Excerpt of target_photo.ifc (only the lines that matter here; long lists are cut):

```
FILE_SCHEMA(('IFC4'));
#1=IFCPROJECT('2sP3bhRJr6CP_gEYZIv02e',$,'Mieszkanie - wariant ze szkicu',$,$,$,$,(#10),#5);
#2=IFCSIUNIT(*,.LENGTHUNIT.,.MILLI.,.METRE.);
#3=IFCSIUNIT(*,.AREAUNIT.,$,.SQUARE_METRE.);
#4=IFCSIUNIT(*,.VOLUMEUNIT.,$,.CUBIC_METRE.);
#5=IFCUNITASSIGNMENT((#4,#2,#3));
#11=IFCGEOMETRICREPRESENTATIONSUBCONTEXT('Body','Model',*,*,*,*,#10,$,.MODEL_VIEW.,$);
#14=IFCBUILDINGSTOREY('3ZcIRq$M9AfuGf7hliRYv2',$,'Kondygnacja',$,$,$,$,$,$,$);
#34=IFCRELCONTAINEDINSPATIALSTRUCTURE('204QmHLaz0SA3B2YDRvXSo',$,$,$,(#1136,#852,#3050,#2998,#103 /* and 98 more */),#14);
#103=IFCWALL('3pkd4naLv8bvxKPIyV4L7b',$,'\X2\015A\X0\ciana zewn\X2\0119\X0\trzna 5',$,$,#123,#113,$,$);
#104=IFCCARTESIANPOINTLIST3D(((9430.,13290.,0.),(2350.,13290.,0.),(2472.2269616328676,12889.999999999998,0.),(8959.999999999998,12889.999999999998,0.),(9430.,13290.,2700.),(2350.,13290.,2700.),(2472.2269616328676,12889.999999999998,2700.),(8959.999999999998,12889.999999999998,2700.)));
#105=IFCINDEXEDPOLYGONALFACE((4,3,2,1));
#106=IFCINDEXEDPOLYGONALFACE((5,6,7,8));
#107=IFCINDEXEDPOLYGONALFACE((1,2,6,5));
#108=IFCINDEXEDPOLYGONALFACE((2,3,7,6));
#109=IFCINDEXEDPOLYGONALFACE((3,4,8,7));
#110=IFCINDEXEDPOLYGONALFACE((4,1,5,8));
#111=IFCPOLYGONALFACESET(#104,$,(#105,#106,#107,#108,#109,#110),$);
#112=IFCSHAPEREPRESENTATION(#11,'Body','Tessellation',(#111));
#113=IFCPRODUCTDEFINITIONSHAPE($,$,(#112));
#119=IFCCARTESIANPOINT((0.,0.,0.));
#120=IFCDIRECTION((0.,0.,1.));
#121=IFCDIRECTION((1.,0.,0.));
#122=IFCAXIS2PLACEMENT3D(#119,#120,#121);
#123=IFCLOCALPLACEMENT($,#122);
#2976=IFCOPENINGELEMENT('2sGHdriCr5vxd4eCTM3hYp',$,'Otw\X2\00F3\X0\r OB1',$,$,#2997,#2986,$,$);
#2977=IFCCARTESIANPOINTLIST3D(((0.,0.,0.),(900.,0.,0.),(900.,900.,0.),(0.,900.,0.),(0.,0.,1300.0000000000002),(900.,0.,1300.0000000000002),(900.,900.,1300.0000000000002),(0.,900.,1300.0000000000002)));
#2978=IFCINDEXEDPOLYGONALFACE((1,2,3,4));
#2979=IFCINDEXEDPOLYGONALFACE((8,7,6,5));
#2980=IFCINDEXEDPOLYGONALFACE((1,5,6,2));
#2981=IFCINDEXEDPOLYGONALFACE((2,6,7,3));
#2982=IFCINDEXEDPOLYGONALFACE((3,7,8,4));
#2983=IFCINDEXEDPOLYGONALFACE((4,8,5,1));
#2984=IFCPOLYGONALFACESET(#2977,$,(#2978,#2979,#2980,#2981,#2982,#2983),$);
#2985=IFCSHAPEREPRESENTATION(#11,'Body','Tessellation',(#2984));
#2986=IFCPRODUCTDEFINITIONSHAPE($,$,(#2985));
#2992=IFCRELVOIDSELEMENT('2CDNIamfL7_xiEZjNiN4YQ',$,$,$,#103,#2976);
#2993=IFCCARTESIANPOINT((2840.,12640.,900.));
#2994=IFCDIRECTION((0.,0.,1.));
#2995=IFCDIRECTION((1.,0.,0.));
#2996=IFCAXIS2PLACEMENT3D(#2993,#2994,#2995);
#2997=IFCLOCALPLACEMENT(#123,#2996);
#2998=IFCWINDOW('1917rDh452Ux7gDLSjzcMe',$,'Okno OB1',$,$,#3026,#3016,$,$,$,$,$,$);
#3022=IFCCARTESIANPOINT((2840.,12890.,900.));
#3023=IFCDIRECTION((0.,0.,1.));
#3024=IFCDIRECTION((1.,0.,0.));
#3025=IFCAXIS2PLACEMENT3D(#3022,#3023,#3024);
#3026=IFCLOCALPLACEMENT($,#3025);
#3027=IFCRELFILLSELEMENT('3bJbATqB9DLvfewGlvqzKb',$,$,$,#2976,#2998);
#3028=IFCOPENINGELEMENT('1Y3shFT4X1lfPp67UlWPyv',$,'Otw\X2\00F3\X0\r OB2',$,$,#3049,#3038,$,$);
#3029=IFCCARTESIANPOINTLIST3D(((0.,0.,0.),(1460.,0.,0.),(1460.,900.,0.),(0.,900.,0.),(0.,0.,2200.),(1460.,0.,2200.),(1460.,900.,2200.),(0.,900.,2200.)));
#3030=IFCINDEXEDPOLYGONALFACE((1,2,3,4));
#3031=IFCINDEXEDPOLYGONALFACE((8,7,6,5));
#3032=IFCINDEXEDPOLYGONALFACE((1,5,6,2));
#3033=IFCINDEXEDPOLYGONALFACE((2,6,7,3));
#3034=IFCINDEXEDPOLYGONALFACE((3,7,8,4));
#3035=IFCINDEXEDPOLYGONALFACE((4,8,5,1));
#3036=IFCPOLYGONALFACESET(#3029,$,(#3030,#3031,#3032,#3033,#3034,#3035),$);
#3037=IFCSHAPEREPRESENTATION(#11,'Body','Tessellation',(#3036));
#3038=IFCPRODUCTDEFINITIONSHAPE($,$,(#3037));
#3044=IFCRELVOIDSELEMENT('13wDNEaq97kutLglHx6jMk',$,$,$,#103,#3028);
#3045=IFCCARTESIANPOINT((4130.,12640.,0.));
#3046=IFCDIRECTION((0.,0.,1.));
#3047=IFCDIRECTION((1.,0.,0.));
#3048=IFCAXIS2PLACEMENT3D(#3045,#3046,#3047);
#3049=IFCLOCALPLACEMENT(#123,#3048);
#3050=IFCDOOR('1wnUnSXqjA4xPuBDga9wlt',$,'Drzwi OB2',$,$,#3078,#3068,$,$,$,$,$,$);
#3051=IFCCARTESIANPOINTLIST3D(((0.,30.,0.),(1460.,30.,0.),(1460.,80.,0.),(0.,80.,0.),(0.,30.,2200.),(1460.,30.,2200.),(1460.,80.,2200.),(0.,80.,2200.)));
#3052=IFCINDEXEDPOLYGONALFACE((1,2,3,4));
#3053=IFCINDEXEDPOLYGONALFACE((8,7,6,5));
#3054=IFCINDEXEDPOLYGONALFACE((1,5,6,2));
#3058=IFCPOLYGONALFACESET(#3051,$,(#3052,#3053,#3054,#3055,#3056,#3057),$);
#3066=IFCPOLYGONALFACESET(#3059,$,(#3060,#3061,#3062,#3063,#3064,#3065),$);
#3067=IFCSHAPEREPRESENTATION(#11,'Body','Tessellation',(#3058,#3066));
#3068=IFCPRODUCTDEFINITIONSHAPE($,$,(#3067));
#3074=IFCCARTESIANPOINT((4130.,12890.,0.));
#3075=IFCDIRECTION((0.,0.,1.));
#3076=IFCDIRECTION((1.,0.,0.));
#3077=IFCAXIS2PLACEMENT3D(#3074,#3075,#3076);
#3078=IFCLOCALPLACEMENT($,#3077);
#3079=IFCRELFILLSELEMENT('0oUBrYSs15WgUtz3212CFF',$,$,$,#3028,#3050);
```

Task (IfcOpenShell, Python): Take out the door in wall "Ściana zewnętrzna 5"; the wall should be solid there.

```python
import ifcopenshell
import ifcopenshell.api.feature
import ifcopenshell.api.root
import ifcopenshell.geom
import ifcopenshell.util.shape

model = ifcopenshell.open("target_photo.ifc")
settings = ifcopenshell.geom.settings()


def volume(element):
    """Net volume in cubic metres, openings subtracted."""
    shape = ifcopenshell.geom.create_shape(settings, element)
    return ifcopenshell.util.shape.get_volume(shape.geometry)


door = model.by_guid("1wnUnSXqjA4xPuBDga9wlt")
opening = door.FillsVoids[0].RelatingOpeningElement
wall = opening.VoidsElements[0].RelatingBuildingElement
before = volume(wall)

ifcopenshell.api.root.remove_product(model, product=door)
ifcopenshell.api.feature.remove_feature(model, feature=opening)

after = volume(wall)

print(f"wall volume {before:.3f} -> {after:.3f} m3")

model.write("target_photo-out.ifc")
```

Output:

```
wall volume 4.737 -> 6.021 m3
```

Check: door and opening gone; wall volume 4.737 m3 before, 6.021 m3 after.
